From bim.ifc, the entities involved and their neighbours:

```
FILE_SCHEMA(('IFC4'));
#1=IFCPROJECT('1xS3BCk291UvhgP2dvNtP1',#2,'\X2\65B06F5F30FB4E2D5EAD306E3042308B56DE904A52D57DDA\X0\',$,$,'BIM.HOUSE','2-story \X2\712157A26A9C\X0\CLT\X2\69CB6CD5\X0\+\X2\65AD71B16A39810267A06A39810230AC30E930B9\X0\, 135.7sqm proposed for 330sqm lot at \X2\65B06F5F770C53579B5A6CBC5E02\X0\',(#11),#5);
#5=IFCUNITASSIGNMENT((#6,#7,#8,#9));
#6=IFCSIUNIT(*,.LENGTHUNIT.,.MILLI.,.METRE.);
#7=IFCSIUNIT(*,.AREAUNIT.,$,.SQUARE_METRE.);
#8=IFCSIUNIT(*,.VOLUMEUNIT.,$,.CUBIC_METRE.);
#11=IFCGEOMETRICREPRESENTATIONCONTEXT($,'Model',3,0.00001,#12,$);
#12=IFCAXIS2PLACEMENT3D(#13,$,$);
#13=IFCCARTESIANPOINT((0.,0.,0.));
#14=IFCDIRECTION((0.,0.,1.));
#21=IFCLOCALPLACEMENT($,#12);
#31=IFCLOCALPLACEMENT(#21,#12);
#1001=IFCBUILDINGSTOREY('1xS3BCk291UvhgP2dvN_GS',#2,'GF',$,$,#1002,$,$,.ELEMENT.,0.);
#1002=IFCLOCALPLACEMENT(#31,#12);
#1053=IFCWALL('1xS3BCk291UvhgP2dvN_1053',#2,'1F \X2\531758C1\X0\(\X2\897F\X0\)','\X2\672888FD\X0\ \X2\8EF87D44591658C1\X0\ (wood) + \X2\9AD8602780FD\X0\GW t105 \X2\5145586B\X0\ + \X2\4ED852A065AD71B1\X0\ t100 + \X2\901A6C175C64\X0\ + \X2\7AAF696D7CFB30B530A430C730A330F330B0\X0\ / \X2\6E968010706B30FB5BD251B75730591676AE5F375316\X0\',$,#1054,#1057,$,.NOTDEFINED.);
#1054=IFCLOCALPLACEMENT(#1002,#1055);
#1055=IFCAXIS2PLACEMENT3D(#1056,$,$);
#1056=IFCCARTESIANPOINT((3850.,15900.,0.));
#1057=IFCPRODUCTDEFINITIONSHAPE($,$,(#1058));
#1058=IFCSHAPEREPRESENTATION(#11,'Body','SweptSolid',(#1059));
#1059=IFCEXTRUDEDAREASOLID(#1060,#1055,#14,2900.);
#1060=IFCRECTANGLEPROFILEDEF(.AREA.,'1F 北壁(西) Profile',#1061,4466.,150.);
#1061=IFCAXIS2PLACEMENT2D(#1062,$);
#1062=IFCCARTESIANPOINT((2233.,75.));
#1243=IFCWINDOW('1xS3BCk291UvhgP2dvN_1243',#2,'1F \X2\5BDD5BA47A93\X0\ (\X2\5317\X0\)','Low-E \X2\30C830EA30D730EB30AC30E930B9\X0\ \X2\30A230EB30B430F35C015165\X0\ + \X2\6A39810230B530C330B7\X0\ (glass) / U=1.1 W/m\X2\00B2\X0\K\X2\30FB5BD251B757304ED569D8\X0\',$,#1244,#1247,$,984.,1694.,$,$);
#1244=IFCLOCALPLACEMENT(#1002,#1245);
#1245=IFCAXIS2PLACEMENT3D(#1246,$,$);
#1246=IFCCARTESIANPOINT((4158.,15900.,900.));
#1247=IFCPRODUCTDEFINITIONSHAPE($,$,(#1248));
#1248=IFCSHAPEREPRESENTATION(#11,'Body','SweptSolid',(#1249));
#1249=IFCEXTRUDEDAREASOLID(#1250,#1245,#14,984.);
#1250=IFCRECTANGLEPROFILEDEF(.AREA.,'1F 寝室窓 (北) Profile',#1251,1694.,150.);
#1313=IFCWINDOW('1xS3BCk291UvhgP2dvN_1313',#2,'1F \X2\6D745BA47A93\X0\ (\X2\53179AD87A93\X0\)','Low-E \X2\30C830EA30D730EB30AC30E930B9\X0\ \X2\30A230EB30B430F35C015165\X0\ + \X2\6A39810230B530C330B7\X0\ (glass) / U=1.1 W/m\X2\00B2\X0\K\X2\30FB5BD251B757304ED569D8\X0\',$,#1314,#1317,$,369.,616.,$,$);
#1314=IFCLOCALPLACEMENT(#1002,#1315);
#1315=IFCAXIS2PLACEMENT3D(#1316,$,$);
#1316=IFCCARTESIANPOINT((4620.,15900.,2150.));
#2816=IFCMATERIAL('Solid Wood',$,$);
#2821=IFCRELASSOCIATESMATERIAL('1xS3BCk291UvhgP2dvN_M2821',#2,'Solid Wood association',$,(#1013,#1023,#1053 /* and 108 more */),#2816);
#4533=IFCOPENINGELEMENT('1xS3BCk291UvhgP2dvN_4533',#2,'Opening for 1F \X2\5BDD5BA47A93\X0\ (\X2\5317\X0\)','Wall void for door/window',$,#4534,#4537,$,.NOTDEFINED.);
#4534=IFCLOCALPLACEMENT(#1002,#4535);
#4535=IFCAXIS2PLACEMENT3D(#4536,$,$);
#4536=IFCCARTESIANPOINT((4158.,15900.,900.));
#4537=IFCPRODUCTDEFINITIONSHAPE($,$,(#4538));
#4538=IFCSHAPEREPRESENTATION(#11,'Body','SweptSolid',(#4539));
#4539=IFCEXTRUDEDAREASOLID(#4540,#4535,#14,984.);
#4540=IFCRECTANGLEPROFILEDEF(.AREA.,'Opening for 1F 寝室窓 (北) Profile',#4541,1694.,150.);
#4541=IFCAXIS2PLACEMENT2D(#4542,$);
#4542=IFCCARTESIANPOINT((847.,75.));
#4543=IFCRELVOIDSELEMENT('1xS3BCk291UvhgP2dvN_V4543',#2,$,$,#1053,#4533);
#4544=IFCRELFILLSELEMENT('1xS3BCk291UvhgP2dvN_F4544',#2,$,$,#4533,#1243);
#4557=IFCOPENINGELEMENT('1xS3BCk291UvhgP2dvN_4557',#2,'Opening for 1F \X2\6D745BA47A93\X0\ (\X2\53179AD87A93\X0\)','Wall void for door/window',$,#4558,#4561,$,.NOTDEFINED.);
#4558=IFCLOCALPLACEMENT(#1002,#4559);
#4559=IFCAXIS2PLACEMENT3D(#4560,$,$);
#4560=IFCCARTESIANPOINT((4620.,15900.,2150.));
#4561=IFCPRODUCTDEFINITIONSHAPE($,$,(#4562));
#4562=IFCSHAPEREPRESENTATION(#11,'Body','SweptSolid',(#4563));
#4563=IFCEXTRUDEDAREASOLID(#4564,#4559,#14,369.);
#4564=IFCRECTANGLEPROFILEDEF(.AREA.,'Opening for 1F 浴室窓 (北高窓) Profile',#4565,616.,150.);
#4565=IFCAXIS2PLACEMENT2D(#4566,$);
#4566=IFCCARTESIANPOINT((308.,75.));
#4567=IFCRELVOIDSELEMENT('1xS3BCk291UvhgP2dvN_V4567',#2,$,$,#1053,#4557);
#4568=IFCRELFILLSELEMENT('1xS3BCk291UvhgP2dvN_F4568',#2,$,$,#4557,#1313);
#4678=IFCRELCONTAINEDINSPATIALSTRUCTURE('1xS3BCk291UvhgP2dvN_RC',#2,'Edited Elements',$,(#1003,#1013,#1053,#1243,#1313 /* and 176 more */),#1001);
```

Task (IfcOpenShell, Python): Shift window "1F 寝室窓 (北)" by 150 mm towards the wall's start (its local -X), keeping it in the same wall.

```python
import ifcopenshell
import ifcopenshell.api.geometry
import ifcopenshell.util.placement
import ifcopenshell.util.unit

model = ifcopenshell.open("bim.ifc")
unit_scale = ifcopenshell.util.unit.calculate_unit_scale(model)

window = model.by_guid("1xS3BCk291UvhgP2dvN_1243")
opening = window.FillsVoids[0].RelatingOpeningElement
wall = opening.VoidsElements[0].RelatingBuildingElement

wall_matrix = ifcopenshell.util.placement.get_local_placement(wall.ObjectPlacement)
shift = wall_matrix[:3, 0] * -0.15 / unit_scale
before = ifcopenshell.util.placement.get_local_placement(window.ObjectPlacement)[:3, 3].copy()

# The window is not placed relative to its opening, so move both.
for product in (opening, window):
    matrix = ifcopenshell.util.placement.get_local_placement(product.ObjectPlacement)
    matrix[:3, 3] += shift
    ifcopenshell.api.geometry.edit_object_placement(model, product=product, matrix=matrix, is_si=False)

after = ifcopenshell.util.placement.get_local_placement(window.ObjectPlacement)[:3, 3]
print("window moved by", (after - before).round(3) + 0.0)

model.write("bim_updated.ifc")
```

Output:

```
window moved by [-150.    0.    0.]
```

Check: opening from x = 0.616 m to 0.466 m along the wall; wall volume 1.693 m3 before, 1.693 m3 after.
